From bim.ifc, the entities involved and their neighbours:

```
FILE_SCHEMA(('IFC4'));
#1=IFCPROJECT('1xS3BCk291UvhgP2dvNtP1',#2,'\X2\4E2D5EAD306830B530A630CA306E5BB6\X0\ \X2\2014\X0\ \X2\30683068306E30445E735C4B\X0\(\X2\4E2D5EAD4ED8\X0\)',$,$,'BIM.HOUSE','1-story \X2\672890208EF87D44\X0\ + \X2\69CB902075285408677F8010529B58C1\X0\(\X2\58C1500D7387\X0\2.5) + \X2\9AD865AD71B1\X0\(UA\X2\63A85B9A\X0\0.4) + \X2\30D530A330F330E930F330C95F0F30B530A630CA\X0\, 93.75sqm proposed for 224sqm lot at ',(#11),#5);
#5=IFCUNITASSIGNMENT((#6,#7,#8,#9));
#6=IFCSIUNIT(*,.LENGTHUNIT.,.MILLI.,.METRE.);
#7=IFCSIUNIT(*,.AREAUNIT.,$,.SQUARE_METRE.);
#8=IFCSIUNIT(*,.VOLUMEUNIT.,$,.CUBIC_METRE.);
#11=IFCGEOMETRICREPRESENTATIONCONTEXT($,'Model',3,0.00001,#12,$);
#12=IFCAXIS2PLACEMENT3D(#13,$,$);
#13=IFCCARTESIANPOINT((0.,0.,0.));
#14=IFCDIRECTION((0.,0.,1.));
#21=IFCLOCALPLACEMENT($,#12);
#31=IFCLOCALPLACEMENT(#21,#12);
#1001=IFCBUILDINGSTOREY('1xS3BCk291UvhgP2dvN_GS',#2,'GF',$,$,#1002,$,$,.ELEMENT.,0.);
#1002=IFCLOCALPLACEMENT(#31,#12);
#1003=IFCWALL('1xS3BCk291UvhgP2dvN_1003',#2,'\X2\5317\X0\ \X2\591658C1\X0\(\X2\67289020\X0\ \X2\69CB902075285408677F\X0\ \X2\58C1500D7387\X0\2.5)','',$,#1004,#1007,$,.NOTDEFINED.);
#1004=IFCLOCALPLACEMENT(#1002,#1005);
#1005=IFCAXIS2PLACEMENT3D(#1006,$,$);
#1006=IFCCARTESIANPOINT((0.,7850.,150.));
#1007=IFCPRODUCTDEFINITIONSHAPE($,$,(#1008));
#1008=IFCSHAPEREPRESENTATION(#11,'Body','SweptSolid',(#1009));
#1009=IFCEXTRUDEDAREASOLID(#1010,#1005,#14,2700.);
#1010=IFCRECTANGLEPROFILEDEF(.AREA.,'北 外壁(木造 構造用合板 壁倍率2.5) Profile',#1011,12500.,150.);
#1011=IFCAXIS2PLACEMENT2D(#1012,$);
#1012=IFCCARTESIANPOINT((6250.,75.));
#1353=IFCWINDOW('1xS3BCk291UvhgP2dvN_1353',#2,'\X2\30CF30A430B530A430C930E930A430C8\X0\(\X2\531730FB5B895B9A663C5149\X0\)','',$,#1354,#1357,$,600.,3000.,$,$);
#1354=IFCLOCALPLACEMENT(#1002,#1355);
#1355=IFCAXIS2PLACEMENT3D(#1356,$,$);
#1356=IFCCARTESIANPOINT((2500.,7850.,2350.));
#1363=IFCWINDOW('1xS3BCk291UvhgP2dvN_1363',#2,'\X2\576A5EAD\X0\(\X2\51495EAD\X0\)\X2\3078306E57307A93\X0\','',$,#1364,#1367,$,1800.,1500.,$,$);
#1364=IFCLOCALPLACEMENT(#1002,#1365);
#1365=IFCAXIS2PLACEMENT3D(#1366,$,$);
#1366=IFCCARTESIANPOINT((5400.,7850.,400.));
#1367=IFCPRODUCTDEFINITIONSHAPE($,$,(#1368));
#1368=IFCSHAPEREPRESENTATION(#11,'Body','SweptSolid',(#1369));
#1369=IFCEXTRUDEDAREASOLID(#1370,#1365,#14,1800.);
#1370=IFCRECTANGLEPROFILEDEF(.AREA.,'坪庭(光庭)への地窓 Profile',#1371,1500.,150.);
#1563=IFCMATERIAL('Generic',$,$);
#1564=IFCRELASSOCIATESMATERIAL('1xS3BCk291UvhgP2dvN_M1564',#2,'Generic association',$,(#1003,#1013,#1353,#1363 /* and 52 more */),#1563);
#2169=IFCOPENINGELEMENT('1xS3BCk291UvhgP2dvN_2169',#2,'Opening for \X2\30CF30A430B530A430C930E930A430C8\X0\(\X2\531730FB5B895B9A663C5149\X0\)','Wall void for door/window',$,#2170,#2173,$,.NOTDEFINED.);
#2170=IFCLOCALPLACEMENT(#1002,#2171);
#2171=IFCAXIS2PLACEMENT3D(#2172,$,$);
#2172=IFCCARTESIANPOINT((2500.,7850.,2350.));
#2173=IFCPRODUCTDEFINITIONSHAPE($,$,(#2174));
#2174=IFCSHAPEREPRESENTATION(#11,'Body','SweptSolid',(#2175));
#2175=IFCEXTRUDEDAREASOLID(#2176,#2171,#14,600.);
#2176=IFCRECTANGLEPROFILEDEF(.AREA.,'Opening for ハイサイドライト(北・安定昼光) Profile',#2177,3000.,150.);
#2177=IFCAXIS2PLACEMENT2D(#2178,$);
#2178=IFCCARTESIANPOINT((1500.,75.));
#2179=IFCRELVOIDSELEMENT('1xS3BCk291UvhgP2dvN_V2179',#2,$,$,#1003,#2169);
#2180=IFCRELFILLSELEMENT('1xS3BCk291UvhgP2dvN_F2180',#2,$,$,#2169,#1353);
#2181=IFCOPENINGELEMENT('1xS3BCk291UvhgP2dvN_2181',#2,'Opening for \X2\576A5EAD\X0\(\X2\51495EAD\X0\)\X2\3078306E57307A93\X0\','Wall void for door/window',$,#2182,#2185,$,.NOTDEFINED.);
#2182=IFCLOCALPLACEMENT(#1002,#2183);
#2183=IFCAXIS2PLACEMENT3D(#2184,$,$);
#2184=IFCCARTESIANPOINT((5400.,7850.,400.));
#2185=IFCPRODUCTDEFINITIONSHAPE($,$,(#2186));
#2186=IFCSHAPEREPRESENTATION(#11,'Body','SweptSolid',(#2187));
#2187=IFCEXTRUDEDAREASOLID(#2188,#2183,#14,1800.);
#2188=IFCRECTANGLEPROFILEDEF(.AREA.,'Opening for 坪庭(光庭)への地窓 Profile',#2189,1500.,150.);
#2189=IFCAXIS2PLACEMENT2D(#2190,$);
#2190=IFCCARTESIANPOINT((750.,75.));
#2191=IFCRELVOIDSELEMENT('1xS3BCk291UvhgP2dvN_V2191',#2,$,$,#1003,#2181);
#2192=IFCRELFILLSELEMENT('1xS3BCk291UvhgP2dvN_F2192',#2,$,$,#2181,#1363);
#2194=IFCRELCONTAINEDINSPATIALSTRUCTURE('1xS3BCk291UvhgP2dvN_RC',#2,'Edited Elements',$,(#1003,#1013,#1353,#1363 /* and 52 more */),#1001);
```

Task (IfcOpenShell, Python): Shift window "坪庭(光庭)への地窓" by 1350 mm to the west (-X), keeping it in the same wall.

```python
import ifcopenshell
import ifcopenshell.api.geometry
import ifcopenshell.util.placement
import ifcopenshell.util.unit

model = ifcopenshell.open("bim.ifc")
unit_scale = ifcopenshell.util.unit.calculate_unit_scale(model)

window = model.by_guid("1xS3BCk291UvhgP2dvN_1363")
opening = window.FillsVoids[0].RelatingOpeningElement
wall = opening.VoidsElements[0].RelatingBuildingElement

wall_matrix = ifcopenshell.util.placement.get_local_placement(wall.ObjectPlacement)
shift = wall_matrix[:3, 0] * -1.35 / unit_scale
before = ifcopenshell.util.placement.get_local_placement(window.ObjectPlacement)[:3, 3].copy()

# The window is not placed relative to its opening, so move both.
for product in (opening, window):
    matrix = ifcopenshell.util.placement.get_local_placement(product.ObjectPlacement)
    matrix[:3, 3] += shift
    ifcopenshell.api.geometry.edit_object_placement(model, product=product, matrix=matrix, is_si=False)

after = ifcopenshell.util.placement.get_local_placement(window.ObjectPlacement)[:3, 3]
print("window moved by", (after - before).round(3) + 0.0)

model.write("bim-out.ifc")
```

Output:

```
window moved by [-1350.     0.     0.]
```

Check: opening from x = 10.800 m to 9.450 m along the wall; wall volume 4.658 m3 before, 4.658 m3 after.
